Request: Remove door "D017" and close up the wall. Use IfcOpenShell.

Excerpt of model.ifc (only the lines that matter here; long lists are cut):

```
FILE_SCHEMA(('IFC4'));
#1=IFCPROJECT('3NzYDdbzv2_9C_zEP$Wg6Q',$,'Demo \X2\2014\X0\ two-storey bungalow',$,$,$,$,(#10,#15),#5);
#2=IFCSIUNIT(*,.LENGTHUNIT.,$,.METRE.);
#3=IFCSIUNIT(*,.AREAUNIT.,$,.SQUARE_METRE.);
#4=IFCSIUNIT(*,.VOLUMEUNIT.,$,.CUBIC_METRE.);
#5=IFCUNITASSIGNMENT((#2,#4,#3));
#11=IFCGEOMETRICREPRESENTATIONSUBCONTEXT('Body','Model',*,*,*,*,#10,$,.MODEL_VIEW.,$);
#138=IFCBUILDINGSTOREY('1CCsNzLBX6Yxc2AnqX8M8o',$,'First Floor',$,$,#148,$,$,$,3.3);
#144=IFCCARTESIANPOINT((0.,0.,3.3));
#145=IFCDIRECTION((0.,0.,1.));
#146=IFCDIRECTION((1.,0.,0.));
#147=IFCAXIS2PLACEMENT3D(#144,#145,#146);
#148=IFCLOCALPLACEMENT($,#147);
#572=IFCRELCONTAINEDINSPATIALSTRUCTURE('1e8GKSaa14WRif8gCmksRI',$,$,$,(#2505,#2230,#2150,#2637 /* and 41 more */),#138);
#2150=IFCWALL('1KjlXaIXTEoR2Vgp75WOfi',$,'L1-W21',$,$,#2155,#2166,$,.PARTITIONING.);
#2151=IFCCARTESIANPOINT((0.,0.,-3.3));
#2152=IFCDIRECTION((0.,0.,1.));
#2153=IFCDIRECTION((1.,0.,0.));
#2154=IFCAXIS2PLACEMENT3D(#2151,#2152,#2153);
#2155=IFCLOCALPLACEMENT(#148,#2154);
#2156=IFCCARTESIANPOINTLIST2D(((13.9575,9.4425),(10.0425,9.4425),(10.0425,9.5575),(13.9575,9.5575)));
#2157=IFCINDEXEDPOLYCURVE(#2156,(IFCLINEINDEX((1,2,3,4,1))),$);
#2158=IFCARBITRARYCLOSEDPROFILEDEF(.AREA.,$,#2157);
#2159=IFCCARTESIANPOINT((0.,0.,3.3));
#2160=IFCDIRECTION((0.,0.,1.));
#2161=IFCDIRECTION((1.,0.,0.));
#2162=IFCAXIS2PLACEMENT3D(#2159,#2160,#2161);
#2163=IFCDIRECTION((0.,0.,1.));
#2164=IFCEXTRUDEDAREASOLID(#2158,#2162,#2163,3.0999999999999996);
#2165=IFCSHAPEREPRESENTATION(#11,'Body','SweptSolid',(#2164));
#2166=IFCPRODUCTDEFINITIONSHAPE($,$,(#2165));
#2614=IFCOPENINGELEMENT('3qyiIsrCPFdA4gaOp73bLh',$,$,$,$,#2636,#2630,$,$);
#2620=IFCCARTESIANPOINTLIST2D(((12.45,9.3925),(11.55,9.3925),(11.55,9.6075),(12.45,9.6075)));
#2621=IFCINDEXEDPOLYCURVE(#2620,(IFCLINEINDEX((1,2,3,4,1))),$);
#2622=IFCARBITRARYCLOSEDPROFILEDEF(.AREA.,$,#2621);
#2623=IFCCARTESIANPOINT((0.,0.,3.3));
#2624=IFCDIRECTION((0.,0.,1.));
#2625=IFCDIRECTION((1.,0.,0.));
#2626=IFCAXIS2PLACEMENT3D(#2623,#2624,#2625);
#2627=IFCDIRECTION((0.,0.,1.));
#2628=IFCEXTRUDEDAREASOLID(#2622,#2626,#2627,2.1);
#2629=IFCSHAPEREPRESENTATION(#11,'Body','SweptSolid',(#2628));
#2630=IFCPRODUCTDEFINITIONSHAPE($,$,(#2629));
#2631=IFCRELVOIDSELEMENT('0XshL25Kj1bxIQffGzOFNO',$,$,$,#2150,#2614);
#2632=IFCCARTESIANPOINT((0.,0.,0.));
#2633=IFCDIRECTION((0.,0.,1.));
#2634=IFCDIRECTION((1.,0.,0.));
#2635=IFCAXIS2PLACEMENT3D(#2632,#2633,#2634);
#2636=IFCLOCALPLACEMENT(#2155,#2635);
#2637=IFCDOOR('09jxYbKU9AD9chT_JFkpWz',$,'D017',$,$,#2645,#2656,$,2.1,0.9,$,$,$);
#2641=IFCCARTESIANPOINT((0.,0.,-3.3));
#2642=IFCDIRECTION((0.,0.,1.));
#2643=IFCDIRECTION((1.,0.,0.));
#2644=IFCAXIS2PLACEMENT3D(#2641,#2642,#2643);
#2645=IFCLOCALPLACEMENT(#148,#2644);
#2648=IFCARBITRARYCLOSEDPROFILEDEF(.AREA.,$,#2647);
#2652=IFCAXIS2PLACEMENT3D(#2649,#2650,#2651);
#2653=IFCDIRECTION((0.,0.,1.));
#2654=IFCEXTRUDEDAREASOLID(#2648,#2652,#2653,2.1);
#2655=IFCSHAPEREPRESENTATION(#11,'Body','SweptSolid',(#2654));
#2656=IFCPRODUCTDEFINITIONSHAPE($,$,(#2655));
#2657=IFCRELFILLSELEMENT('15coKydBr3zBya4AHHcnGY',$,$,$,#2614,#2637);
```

```python
import ifcopenshell
import ifcopenshell.api.feature
import ifcopenshell.api.root
import ifcopenshell.geom
import ifcopenshell.util.shape

model = ifcopenshell.open("model.ifc")
settings = ifcopenshell.geom.settings()


def volume(element):
    """Net volume in cubic metres, openings subtracted."""
    shape = ifcopenshell.geom.create_shape(settings, element)
    return ifcopenshell.util.shape.get_volume(shape.geometry)


door = model.by_id(2637)
opening = door.FillsVoids[0].RelatingOpeningElement
wall = opening.VoidsElements[0].RelatingBuildingElement
before = volume(wall)

ifcopenshell.api.root.remove_product(model, product=door)
ifcopenshell.api.feature.remove_feature(model, feature=opening)

after = volume(wall)

print(f"wall volume {before:.3f} -> {after:.3f} m3")

model.write("model_updated.ifc")
```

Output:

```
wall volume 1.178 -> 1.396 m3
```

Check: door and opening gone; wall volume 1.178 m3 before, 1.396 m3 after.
